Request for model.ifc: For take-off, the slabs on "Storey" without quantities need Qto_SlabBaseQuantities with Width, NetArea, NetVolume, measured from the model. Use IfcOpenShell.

First a look at what the model holds.

```python
import ifcopenshell
import ifcopenshell.util.element
import ifcopenshell.util.unit

model = ifcopenshell.open("model.ifc")
print(model.schema)
for unit_type in ("LENGTHUNIT", "AREAUNIT", "VOLUMEUNIT"):
    print(unit_type, ifcopenshell.util.unit.calculate_unit_scale(model, unit_type))
storey = next(s for s in model.by_type("IfcBuildingStorey") if s.Name == "Storey")
slabs = [e for e in ifcopenshell.util.element.get_decomposition(storey) if e.is_a("IfcSlab")]
for e in sorted(slabs, key=lambda e: e.id()):
    print(e.id(), e.is_a(), e.Name, list(ifcopenshell.util.element.get_psets(e, qtos_only=True)), sep=" | ")
```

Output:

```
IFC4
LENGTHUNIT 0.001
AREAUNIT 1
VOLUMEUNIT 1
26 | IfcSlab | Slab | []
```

```python
import ifcopenshell
import ifcopenshell.api.pset
import ifcopenshell.geom
import ifcopenshell.util.element
import ifcopenshell.util.shape
import ifcopenshell.util.unit

model = ifcopenshell.open("model.ifc")
unit_scale = ifcopenshell.util.unit.calculate_unit_scale(model)
area_scale = ifcopenshell.util.unit.calculate_unit_scale(model, "AREAUNIT")
volume_scale = ifcopenshell.util.unit.calculate_unit_scale(model, "VOLUMEUNIT")
settings = ifcopenshell.geom.settings()

storey = next(s for s in model.by_type("IfcBuildingStorey") if s.Name == "Storey")
slabs = [e for e in ifcopenshell.util.element.get_decomposition(storey) if e.is_a("IfcSlab")]

for e in sorted(slabs, key=lambda e: e.id()):
    if ifcopenshell.util.element.get_psets(e, qtos_only=True, should_inherit=False):
        continue
    # Geometry comes back in metres, in the element's own axes.
    shape = ifcopenshell.geom.create_shape(settings, e)
    values = {
        "Width": ifcopenshell.util.shape.get_z(shape.geometry) / unit_scale,
        "NetArea": ifcopenshell.util.shape.get_footprint_area(shape.geometry) / area_scale,
        "NetVolume": ifcopenshell.util.shape.get_volume(shape.geometry) / volume_scale,
    }
    qto = ifcopenshell.api.pset.add_qto(model, product=e, name="Qto_SlabBaseQuantities")
    ifcopenshell.api.pset.edit_qto(model, qto=qto, properties=values)
    print(e.id(), {k: round(v, 3) for k, v in values.items()})

model.write("model_v2.ifc")
```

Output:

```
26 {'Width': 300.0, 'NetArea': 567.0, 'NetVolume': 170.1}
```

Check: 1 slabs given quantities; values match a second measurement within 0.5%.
